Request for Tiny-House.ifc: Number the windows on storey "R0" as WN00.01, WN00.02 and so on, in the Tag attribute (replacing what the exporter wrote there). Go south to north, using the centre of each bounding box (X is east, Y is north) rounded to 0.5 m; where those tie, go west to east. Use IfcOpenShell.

First a look at what the model holds.

```python
import ifcopenshell
import ifcopenshell.util.element
import ifcopenshell.util.placement

model = ifcopenshell.open("Tiny-House.ifc")
print(model.schema)
storey = next(s for s in model.by_type("IfcBuildingStorey") if s.Name == "R0")
windows = [e for e in ifcopenshell.util.element.get_decomposition(storey) if e.is_a("IfcWindow")]
for e in sorted(windows, key=lambda e: e.id()):
    origin = ifcopenshell.util.placement.get_local_placement(e.ObjectPlacement)[:3, 3]
    print(e.id(), e.Tag, e.Name, origin.round(2) + 0.0, sep=" | ")
```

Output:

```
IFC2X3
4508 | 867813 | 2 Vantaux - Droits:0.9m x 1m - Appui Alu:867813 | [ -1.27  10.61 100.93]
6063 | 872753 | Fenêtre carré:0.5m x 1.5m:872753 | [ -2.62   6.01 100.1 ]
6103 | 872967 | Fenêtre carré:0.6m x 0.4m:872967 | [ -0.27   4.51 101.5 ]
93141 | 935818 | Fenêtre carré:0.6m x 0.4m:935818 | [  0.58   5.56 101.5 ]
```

```python
import ifcopenshell
import ifcopenshell.geom
import ifcopenshell.util.element
import ifcopenshell.util.shape

model = ifcopenshell.open("Tiny-House.ifc")
settings = ifcopenshell.geom.settings()
settings.set("use-world-coords", True)


def centre(element):
    shape = ifcopenshell.geom.create_shape(settings, element)
    return ifcopenshell.util.shape.get_bbox_centroid(shape.geometry)


storey = next(s for s in model.by_type("IfcBuildingStorey") if s.Name == "R0")
windows = [e for e in ifcopenshell.util.element.get_decomposition(storey) if e.is_a("IfcWindow")]

# Insertion points can sit at a corner or the storey origin, so sort by the geometry (in metres).
centres = {e: centre(e) for e in windows}
windows.sort(key=lambda e: (round(centres[e][1] / 0.5), centres[e][0]))

for i, e in enumerate(windows, start=1):
    number = f"WN00.{i:02d}"
    e.Tag = number
    print(e.id(), number)

model.write("Tiny-House_updated.ifc")
```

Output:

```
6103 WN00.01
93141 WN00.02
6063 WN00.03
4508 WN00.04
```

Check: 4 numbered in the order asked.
